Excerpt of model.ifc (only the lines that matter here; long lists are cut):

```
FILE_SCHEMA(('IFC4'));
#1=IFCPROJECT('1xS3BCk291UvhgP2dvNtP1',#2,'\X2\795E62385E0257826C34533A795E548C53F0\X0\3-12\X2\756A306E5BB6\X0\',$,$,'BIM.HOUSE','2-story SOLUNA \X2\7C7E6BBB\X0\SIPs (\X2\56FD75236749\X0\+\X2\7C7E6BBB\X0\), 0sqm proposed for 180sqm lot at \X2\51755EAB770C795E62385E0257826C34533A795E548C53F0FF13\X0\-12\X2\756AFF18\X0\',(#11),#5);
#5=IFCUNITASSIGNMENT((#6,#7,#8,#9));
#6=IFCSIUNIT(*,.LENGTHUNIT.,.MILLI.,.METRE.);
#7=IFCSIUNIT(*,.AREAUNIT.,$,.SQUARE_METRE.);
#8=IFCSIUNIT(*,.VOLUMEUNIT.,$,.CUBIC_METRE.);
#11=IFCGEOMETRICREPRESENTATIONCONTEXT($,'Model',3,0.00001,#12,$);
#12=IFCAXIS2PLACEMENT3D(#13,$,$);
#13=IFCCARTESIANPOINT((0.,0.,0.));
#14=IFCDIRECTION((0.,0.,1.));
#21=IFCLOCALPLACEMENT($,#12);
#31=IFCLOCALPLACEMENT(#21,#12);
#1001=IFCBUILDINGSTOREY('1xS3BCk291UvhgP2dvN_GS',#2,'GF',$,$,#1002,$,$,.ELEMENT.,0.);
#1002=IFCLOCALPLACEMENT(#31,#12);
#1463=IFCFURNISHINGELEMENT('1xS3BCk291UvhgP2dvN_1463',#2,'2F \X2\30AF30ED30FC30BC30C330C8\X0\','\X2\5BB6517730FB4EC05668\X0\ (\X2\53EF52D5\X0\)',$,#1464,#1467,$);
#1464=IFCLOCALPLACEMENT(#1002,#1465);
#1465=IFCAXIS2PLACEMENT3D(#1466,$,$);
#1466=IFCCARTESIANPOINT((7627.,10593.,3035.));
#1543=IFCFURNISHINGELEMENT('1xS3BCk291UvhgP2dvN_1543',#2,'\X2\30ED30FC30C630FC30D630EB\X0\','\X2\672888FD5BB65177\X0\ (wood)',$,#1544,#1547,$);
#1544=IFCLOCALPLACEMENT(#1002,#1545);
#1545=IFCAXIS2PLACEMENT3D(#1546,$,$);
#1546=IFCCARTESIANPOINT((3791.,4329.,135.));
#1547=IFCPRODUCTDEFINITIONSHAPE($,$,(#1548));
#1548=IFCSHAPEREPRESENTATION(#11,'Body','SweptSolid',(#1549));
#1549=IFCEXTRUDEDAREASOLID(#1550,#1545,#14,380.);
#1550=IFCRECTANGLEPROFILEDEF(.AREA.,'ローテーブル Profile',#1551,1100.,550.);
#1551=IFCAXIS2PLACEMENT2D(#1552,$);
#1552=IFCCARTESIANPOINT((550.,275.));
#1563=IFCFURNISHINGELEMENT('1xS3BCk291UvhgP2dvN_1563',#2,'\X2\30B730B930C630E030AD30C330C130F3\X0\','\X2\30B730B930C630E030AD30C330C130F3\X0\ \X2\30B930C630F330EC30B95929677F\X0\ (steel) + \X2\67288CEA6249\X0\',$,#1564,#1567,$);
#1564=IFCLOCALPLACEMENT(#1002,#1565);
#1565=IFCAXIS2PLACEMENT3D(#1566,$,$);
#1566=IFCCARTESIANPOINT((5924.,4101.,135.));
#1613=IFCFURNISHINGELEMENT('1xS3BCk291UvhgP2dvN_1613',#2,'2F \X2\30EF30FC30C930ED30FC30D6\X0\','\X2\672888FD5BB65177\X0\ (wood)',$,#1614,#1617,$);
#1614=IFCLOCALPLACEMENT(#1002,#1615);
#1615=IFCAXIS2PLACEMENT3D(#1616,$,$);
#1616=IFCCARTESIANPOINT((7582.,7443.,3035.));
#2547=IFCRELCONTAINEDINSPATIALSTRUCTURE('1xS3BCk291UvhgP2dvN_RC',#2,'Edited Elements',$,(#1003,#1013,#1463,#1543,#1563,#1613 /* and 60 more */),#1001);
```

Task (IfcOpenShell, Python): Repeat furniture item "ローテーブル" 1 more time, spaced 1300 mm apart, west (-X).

```python
import numpy as np
import ifcopenshell
import ifcopenshell.api.geometry
import ifcopenshell.api.root
import ifcopenshell.util.element
import ifcopenshell.util.placement

model = ifcopenshell.open("model.ifc")


def reuse_history(source, copy):
    """copy_class also copies each property set's owner history, people and application; keep the originals."""
    for rel in copy.IsDefinedBy:
        if rel.is_a("IfcRelDefinesByProperties") and (history := rel.RelatingPropertyDefinition.OwnerHistory):
            rel.RelatingPropertyDefinition.OwnerHistory = source.OwnerHistory
            ifcopenshell.util.element.remove_deep2(model, history)


source = model.by_guid("1xS3BCk291UvhgP2dvN_1543")
base = ifcopenshell.util.placement.get_local_placement(source.ObjectPlacement)
step = np.array([-1.0, 0.0, 0.0]) * 1300.0

for i in range(1, 2):
    copy = ifcopenshell.api.root.copy_class(model, product=source)
    copy.Representation = ifcopenshell.util.element.copy_deep(
        model, source.Representation, exclude=["IfcGeometricRepresentationContext", "IfcRepresentationMap"]
    )
    reuse_history(source, copy)
    matrix = base.copy()
    matrix[:3, 3] += i * step
    print("added at", matrix[:3, 3].round(3) + 0.0)
    ifcopenshell.api.geometry.edit_object_placement(model, product=copy, matrix=matrix, is_si=False)

model.write("model_edited.ifc")
```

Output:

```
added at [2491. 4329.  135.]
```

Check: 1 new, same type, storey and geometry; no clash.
